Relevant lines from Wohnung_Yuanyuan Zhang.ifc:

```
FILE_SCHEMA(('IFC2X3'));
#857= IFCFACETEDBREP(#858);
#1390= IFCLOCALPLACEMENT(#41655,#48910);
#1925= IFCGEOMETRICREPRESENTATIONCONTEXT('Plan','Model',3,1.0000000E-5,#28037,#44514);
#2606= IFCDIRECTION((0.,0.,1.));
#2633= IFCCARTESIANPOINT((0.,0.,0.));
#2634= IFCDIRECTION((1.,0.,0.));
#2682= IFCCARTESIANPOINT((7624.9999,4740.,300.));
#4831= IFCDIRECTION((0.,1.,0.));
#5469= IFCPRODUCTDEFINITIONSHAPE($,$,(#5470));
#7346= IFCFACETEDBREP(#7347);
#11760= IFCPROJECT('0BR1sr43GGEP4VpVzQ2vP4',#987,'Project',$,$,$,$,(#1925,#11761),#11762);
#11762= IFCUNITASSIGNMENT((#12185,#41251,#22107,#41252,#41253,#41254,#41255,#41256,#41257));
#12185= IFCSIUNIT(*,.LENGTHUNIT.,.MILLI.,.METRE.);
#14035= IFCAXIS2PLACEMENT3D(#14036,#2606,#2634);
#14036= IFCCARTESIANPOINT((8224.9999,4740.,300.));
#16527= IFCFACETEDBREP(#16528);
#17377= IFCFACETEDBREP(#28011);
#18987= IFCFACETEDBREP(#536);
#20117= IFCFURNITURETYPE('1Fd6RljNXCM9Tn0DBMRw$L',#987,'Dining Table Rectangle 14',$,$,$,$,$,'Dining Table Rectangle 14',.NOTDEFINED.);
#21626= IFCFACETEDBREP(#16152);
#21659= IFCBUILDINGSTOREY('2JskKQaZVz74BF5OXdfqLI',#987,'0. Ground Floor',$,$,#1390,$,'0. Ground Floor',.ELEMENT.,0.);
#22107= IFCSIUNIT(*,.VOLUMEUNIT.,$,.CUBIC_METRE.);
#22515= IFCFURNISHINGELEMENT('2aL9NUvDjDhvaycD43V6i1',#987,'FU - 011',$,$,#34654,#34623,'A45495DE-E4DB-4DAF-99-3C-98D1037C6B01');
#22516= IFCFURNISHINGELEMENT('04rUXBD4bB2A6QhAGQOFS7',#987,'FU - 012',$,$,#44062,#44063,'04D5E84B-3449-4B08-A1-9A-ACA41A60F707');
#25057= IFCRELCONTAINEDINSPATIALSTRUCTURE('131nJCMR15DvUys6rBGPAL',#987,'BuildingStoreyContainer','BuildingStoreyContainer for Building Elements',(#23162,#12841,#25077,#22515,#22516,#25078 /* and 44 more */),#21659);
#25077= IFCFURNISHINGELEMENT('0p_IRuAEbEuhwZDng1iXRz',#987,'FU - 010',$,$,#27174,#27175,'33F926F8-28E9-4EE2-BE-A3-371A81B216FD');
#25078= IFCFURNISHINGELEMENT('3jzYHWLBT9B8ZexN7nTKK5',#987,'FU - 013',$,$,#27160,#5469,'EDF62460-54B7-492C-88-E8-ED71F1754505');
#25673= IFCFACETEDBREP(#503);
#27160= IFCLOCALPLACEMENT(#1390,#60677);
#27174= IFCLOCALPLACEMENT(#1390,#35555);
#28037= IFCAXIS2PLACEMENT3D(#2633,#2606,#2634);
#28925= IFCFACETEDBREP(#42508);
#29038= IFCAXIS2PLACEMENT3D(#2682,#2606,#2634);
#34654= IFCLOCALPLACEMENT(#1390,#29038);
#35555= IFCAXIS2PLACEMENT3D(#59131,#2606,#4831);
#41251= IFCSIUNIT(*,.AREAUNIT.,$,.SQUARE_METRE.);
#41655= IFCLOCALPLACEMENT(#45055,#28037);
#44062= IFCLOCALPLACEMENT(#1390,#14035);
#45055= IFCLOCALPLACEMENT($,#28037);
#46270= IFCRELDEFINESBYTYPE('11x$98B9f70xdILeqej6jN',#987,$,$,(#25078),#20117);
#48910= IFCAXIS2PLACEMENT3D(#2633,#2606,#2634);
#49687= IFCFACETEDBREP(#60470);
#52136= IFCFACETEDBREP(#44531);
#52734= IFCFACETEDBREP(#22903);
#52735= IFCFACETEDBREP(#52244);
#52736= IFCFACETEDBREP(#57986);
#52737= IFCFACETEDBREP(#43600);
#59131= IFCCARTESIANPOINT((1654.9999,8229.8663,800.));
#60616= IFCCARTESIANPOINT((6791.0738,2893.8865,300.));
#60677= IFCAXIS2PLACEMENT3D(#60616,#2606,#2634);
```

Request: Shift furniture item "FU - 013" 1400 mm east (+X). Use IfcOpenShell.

```python
import ifcopenshell
import ifcopenshell.api.geometry
import ifcopenshell.util.placement
import ifcopenshell.util.unit

model = ifcopenshell.open("Wohnung_Yuanyuan Zhang.ifc")
unit_scale = ifcopenshell.util.unit.calculate_unit_scale(model)

item = model.by_id(25078)
matrix = ifcopenshell.util.placement.get_local_placement(item.ObjectPlacement)
matrix[0, 3] += 1.4 / unit_scale
ifcopenshell.api.geometry.edit_object_placement(model, product=item, matrix=matrix, is_si=False)

print(ifcopenshell.util.placement.get_local_placement(item.ObjectPlacement).round(3) + 0.0)

model.write("Wohnung_Yuanyuan Zhang-out.ifc")
```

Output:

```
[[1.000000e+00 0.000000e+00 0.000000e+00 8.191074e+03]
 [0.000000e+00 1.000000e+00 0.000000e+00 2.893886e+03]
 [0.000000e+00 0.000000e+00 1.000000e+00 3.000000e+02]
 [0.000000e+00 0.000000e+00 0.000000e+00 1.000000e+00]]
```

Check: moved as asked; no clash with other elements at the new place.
